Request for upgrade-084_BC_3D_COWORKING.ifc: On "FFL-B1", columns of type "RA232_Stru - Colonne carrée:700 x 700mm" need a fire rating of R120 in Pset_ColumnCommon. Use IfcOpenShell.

First a look at what the model holds.

```python
import ifcopenshell
import ifcopenshell.util.element

model = ifcopenshell.open("upgrade-084_BC_3D_COWORKING.ifc")
print(model.schema)
storey = next(s for s in model.by_type("IfcBuildingStorey") if s.Name == "FFL-B1")
columns = [e for e in ifcopenshell.util.element.get_decomposition(storey) if e.is_a("IfcColumn")]
seen = {}
for e in columns:
    element_type = ifcopenshell.util.element.get_type(e)
    key = (element_type.Name if element_type != e and element_type else None, ifcopenshell.util.element.get_pset(e, "Pset_ColumnCommon", "FireRating"))
    seen[key] = seen.get(key, 0) + 1
for (name, value), count in sorted(seen.items(), key=str):
    print(count, "x", name, "|", value)
```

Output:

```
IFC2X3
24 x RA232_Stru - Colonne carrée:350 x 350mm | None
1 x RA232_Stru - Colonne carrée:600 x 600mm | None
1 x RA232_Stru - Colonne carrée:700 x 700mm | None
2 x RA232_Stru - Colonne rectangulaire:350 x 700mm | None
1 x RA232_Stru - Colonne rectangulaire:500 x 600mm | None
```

```python
import ifcopenshell
import ifcopenshell.api.pset
import ifcopenshell.util.element

model = ifcopenshell.open("upgrade-084_BC_3D_COWORKING.ifc")

storey = next(s for s in model.by_type("IfcBuildingStorey") if s.Name == "FFL-B1")
columns = [e for e in ifcopenshell.util.element.get_decomposition(storey) if e.is_a("IfcColumn")]

count = 0
for e in columns:
    element_type = ifcopenshell.util.element.get_type(e)
    if element_type in (None, e) or element_type.Name != "RA232_Stru - Colonne carrée:700 x 700mm":
        continue
    # add_pset returns the element's existing set when there is one.
    pset = ifcopenshell.api.pset.add_pset(model, product=e, name="Pset_ColumnCommon")
    ifcopenshell.api.pset.edit_pset(model, pset=pset, properties={"FireRating": "R120"})
    count += 1

print(count, "columns updated")

model.write("upgrade-084_BC_3D_COWORKING_edited.ifc")
```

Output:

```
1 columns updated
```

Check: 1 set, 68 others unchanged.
